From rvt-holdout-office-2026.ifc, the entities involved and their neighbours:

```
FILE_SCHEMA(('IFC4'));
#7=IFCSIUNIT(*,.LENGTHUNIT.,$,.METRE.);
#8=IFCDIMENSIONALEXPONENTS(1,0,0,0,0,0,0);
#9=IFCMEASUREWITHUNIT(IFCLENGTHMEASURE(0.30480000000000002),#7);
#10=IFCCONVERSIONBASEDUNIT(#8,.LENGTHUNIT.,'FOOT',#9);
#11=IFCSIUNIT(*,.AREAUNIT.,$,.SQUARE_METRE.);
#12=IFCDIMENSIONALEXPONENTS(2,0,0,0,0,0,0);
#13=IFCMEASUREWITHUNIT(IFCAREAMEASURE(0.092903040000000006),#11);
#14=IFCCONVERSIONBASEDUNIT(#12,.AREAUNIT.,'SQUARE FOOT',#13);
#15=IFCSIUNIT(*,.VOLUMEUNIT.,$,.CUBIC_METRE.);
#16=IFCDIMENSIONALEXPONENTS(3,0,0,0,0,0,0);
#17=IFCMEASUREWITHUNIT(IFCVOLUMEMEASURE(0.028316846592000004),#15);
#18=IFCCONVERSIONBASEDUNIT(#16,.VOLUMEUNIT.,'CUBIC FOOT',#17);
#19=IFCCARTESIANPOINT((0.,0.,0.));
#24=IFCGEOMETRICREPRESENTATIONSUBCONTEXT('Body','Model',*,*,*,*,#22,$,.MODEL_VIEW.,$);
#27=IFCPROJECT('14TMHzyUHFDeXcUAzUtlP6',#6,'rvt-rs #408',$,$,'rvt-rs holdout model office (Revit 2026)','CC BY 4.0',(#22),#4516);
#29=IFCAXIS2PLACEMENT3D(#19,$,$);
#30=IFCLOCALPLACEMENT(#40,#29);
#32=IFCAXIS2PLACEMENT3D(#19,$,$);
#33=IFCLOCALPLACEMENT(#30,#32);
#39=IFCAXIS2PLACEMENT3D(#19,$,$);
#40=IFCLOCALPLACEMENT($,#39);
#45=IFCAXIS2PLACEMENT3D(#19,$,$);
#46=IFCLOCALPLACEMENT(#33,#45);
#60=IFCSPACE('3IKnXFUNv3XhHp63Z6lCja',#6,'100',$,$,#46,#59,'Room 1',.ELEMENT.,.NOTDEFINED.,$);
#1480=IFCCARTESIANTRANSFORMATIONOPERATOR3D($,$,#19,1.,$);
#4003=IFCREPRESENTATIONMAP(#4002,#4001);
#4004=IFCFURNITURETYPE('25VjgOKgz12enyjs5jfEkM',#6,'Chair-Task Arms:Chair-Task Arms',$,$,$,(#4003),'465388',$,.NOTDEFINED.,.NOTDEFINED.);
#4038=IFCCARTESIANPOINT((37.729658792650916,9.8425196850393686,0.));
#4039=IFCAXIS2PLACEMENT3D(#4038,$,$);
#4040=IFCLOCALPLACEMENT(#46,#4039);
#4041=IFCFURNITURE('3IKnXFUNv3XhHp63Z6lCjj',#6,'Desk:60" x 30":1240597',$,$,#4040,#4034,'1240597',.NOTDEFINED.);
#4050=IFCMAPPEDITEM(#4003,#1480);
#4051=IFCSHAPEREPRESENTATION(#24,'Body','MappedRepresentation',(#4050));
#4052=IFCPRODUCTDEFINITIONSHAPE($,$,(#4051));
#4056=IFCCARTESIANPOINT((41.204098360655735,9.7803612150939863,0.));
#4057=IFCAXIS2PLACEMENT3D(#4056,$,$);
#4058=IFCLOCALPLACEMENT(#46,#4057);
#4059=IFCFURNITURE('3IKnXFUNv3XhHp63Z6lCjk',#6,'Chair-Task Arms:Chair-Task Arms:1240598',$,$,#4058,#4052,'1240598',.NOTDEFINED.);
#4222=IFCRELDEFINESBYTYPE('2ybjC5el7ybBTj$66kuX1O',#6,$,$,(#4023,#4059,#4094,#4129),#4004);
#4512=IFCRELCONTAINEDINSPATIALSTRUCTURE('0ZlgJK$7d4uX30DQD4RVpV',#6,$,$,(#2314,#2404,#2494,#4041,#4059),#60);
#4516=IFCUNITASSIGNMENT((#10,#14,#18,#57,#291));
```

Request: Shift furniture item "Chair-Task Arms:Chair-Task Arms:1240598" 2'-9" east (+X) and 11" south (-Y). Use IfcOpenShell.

```python
import ifcopenshell
import ifcopenshell.api.geometry
import ifcopenshell.util.placement
import ifcopenshell.util.unit

model = ifcopenshell.open("rvt-holdout-office-2026.ifc")
unit_scale = ifcopenshell.util.unit.calculate_unit_scale(model)

item = model.by_guid("3IKnXFUNv3XhHp63Z6lCjk")
matrix = ifcopenshell.util.placement.get_local_placement(item.ObjectPlacement)
matrix[0, 3] += 33 * 0.0254 / unit_scale
matrix[1, 3] -= 11 * 0.0254 / unit_scale
ifcopenshell.api.geometry.edit_object_placement(model, product=item, matrix=matrix, is_si=False)

print(ifcopenshell.util.placement.get_local_placement(item.ObjectPlacement).round(3) + 0.0)

model.write("rvt-holdout-office-2026_rev.ifc")
```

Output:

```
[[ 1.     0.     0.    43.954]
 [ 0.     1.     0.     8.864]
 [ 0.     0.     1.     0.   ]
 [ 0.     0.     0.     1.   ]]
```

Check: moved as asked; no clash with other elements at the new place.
